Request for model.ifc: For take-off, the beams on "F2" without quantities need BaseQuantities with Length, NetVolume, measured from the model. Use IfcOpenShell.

First a look at what the model holds.

```python
import ifcopenshell
import ifcopenshell.util.element
import ifcopenshell.util.unit

model = ifcopenshell.open("model.ifc")
print(model.schema)
for unit_type in ("LENGTHUNIT", "AREAUNIT", "VOLUMEUNIT"):
    print(unit_type, ifcopenshell.util.unit.calculate_unit_scale(model, unit_type))
storey = next(s for s in model.by_type("IfcBuildingStorey") if s.Name == "F2")
beams = [e for e in ifcopenshell.util.element.get_decomposition(storey) if e.is_a("IfcBeam")]
for e in sorted(beams, key=lambda e: e.id()):
    print(e.id(), e.is_a(), e.Name, list(ifcopenshell.util.element.get_psets(e, qtos_only=True)), sep=" | ")
```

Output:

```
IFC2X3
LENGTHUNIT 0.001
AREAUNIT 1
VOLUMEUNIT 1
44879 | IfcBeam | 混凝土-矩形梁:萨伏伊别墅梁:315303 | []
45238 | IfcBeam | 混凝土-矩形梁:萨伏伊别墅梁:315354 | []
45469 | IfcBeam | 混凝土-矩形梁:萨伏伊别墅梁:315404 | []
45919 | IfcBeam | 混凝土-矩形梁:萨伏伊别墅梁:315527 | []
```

```python
import ifcopenshell
import ifcopenshell.api.pset
import ifcopenshell.geom
import ifcopenshell.util.element
import ifcopenshell.util.shape
import ifcopenshell.util.unit

model = ifcopenshell.open("model.ifc")
unit_scale = ifcopenshell.util.unit.calculate_unit_scale(model)
volume_scale = ifcopenshell.util.unit.calculate_unit_scale(model, "VOLUMEUNIT")
settings = ifcopenshell.geom.settings()

storey = next(s for s in model.by_type("IfcBuildingStorey") if s.Name == "F2")
beams = [e for e in ifcopenshell.util.element.get_decomposition(storey) if e.is_a("IfcBeam")]

for e in sorted(beams, key=lambda e: e.id()):
    if ifcopenshell.util.element.get_psets(e, qtos_only=True, should_inherit=False):
        continue
    # Geometry comes back in metres, in the element's own axes.
    shape = ifcopenshell.geom.create_shape(settings, e)
    values = {
        "Length": ifcopenshell.util.shape.get_max_xyz(shape.geometry) / unit_scale,
        "NetVolume": ifcopenshell.util.shape.get_volume(shape.geometry) / volume_scale,
    }
    qto = ifcopenshell.api.pset.add_qto(model, product=e, name="BaseQuantities")
    ifcopenshell.api.pset.edit_qto(model, qto=qto, properties=values)
    print(e.id(), {k: round(v, 3) for k, v in values.items()})

model.write("model_edited.ifc")
```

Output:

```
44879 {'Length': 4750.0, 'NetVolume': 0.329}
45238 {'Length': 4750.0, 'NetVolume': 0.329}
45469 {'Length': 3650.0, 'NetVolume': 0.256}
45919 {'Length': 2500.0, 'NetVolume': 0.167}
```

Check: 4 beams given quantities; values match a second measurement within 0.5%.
